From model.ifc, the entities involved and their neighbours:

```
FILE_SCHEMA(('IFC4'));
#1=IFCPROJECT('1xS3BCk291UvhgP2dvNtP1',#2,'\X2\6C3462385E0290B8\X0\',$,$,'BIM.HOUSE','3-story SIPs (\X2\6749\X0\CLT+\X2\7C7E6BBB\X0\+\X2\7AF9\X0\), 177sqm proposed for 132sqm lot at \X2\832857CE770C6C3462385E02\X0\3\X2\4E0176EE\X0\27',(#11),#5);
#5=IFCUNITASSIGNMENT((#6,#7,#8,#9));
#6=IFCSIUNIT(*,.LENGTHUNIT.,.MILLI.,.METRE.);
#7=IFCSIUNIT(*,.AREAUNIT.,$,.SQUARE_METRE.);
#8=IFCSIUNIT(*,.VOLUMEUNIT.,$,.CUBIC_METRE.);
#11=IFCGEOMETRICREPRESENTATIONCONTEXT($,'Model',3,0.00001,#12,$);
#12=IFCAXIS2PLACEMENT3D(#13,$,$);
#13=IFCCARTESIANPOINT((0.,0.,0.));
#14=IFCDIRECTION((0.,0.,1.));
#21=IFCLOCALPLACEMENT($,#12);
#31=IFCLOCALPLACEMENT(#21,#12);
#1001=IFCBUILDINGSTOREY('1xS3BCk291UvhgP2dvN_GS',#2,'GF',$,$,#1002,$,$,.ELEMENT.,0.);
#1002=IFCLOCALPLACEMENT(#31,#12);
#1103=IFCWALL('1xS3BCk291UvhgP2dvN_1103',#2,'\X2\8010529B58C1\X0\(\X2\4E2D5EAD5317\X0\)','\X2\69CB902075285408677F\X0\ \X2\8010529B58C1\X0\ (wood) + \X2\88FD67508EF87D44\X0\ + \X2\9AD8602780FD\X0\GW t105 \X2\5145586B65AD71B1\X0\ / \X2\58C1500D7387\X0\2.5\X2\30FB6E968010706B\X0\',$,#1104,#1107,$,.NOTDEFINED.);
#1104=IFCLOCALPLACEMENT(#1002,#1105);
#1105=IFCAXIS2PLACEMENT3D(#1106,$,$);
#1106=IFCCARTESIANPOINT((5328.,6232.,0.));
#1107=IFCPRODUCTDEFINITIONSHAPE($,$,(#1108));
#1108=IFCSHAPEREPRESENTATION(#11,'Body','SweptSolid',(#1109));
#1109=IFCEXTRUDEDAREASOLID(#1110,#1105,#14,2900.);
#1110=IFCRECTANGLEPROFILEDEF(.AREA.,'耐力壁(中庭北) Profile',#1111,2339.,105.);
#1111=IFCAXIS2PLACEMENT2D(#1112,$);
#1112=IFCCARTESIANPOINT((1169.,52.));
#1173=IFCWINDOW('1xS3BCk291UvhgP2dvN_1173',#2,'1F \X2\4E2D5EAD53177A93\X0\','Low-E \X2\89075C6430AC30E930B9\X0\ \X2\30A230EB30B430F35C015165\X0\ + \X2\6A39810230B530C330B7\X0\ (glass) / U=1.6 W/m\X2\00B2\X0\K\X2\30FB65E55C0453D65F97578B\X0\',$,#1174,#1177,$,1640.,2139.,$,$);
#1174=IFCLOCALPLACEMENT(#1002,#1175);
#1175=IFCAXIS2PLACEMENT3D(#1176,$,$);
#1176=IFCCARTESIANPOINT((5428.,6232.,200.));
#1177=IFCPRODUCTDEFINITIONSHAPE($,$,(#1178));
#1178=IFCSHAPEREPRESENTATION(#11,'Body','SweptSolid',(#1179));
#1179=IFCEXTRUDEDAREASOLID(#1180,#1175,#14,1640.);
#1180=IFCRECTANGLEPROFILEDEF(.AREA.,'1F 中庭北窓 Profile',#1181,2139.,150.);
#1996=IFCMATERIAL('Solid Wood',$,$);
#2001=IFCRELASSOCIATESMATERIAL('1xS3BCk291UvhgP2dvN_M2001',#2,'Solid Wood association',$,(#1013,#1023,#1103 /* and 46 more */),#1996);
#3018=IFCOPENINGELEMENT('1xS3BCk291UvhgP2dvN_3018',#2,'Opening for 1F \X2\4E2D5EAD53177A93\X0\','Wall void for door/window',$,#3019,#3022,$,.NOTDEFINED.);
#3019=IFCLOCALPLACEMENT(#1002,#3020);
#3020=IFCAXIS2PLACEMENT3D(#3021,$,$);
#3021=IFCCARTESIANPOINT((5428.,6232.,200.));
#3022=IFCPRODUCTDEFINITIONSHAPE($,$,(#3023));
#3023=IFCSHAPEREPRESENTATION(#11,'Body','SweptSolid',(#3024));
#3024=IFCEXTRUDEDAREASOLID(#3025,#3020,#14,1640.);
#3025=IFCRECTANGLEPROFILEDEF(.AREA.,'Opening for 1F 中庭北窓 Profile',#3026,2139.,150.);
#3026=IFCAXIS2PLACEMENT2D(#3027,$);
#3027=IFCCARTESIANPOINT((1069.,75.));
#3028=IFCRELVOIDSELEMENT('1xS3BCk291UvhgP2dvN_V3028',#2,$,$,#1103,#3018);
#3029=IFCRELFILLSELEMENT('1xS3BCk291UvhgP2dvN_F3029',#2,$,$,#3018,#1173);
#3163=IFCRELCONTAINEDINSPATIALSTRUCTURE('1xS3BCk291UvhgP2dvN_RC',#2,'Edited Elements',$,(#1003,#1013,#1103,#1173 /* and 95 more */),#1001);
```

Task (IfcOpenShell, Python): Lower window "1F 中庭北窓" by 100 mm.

```python
import numpy as np
import ifcopenshell
import ifcopenshell.api.geometry
import ifcopenshell.util.placement
import ifcopenshell.util.unit

model = ifcopenshell.open("model.ifc")
unit_scale = ifcopenshell.util.unit.calculate_unit_scale(model)

window = model.by_id(1173)
opening = window.FillsVoids[0].RelatingOpeningElement
dz = -100.0

shift = np.array([0.0, 0.0, dz])
# The window is not placed relative to its opening, so move both.
for product in (opening, window):
    matrix = ifcopenshell.util.placement.get_local_placement(product.ObjectPlacement)
    matrix[:3, 3] += shift
    ifcopenshell.api.geometry.edit_object_placement(model, product=product, matrix=matrix, is_si=False)

print(f"moved by {dz * unit_scale:+.3f} m")

model.write("model_rev.ifc")
```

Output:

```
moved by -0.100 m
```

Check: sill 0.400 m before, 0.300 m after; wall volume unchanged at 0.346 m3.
